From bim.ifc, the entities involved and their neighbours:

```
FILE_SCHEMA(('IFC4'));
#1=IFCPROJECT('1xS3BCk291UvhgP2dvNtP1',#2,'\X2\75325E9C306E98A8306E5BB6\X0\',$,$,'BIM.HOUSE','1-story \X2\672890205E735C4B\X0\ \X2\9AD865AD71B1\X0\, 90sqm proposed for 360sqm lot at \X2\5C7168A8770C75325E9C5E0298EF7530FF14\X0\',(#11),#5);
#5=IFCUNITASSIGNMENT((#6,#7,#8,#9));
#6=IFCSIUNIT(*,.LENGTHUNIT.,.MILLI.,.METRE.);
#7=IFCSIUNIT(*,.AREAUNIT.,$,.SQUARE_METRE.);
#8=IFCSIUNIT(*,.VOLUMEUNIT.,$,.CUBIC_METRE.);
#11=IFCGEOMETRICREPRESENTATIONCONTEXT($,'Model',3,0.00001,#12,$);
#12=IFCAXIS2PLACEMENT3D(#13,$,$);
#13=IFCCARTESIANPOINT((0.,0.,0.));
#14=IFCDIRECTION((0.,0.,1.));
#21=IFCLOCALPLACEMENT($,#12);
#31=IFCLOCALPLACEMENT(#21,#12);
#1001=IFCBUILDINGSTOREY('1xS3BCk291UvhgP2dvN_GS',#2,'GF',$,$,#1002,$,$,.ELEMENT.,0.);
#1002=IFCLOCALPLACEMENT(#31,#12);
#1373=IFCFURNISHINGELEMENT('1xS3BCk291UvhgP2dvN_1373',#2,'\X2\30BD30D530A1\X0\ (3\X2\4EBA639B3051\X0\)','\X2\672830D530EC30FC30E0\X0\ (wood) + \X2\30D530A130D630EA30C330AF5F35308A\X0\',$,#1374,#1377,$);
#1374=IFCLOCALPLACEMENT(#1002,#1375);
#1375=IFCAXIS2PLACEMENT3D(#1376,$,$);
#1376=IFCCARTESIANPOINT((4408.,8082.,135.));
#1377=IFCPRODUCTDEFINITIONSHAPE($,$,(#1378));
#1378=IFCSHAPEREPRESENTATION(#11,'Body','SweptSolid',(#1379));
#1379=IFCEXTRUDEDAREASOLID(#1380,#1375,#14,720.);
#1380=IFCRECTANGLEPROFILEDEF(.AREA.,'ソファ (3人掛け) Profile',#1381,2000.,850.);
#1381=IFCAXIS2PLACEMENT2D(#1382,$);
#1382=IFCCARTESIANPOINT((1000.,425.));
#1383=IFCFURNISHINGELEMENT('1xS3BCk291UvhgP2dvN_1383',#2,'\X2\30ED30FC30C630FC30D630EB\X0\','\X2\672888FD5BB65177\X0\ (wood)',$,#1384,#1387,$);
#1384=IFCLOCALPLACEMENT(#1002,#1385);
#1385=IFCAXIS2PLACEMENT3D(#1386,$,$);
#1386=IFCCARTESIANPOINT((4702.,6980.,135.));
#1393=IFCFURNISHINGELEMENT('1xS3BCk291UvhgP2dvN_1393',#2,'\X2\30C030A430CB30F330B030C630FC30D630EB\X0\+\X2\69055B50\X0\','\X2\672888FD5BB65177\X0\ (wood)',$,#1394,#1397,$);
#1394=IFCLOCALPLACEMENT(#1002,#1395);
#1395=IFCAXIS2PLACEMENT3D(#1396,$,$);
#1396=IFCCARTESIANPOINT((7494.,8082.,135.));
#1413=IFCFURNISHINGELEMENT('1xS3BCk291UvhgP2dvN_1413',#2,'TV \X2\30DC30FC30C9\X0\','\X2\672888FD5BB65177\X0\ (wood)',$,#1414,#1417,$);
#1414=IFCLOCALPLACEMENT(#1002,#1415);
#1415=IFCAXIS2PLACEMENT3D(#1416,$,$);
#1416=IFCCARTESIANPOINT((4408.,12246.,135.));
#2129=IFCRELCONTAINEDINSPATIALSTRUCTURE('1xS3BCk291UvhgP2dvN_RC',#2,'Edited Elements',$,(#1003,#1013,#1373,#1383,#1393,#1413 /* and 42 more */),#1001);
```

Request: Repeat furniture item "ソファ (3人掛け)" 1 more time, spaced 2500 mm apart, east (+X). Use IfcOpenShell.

```python
import numpy as np
import ifcopenshell
import ifcopenshell.api.geometry
import ifcopenshell.api.root
import ifcopenshell.util.element
import ifcopenshell.util.placement
import ifcopenshell.util.unit

model = ifcopenshell.open("bim.ifc")
unit_scale = ifcopenshell.util.unit.calculate_unit_scale(model)


def reuse_history(source, copy):
    """copy_class also copies each property set's owner history, people and application; keep the originals."""
    for rel in copy.IsDefinedBy:
        if rel.is_a("IfcRelDefinesByProperties") and (history := rel.RelatingPropertyDefinition.OwnerHistory):
            rel.RelatingPropertyDefinition.OwnerHistory = source.OwnerHistory
            ifcopenshell.util.element.remove_deep2(model, history)


source = model.by_id(1373)
base = ifcopenshell.util.placement.get_local_placement(source.ObjectPlacement)
step = np.array([1.0, 0.0, 0.0]) * 2.5 / unit_scale

for i in range(1, 2):
    copy = ifcopenshell.api.root.copy_class(model, product=source)
    copy.Representation = ifcopenshell.util.element.copy_deep(
        model, source.Representation, exclude=["IfcGeometricRepresentationContext", "IfcRepresentationMap"]
    )
    reuse_history(source, copy)
    matrix = base.copy()
    matrix[:3, 3] += i * step
    print("added at", matrix[:3, 3].round(3) + 0.0)
    ifcopenshell.api.geometry.edit_object_placement(model, product=copy, matrix=matrix, is_si=False)

model.write("bim_edited.ifc")
```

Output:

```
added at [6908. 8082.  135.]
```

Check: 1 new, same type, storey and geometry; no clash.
